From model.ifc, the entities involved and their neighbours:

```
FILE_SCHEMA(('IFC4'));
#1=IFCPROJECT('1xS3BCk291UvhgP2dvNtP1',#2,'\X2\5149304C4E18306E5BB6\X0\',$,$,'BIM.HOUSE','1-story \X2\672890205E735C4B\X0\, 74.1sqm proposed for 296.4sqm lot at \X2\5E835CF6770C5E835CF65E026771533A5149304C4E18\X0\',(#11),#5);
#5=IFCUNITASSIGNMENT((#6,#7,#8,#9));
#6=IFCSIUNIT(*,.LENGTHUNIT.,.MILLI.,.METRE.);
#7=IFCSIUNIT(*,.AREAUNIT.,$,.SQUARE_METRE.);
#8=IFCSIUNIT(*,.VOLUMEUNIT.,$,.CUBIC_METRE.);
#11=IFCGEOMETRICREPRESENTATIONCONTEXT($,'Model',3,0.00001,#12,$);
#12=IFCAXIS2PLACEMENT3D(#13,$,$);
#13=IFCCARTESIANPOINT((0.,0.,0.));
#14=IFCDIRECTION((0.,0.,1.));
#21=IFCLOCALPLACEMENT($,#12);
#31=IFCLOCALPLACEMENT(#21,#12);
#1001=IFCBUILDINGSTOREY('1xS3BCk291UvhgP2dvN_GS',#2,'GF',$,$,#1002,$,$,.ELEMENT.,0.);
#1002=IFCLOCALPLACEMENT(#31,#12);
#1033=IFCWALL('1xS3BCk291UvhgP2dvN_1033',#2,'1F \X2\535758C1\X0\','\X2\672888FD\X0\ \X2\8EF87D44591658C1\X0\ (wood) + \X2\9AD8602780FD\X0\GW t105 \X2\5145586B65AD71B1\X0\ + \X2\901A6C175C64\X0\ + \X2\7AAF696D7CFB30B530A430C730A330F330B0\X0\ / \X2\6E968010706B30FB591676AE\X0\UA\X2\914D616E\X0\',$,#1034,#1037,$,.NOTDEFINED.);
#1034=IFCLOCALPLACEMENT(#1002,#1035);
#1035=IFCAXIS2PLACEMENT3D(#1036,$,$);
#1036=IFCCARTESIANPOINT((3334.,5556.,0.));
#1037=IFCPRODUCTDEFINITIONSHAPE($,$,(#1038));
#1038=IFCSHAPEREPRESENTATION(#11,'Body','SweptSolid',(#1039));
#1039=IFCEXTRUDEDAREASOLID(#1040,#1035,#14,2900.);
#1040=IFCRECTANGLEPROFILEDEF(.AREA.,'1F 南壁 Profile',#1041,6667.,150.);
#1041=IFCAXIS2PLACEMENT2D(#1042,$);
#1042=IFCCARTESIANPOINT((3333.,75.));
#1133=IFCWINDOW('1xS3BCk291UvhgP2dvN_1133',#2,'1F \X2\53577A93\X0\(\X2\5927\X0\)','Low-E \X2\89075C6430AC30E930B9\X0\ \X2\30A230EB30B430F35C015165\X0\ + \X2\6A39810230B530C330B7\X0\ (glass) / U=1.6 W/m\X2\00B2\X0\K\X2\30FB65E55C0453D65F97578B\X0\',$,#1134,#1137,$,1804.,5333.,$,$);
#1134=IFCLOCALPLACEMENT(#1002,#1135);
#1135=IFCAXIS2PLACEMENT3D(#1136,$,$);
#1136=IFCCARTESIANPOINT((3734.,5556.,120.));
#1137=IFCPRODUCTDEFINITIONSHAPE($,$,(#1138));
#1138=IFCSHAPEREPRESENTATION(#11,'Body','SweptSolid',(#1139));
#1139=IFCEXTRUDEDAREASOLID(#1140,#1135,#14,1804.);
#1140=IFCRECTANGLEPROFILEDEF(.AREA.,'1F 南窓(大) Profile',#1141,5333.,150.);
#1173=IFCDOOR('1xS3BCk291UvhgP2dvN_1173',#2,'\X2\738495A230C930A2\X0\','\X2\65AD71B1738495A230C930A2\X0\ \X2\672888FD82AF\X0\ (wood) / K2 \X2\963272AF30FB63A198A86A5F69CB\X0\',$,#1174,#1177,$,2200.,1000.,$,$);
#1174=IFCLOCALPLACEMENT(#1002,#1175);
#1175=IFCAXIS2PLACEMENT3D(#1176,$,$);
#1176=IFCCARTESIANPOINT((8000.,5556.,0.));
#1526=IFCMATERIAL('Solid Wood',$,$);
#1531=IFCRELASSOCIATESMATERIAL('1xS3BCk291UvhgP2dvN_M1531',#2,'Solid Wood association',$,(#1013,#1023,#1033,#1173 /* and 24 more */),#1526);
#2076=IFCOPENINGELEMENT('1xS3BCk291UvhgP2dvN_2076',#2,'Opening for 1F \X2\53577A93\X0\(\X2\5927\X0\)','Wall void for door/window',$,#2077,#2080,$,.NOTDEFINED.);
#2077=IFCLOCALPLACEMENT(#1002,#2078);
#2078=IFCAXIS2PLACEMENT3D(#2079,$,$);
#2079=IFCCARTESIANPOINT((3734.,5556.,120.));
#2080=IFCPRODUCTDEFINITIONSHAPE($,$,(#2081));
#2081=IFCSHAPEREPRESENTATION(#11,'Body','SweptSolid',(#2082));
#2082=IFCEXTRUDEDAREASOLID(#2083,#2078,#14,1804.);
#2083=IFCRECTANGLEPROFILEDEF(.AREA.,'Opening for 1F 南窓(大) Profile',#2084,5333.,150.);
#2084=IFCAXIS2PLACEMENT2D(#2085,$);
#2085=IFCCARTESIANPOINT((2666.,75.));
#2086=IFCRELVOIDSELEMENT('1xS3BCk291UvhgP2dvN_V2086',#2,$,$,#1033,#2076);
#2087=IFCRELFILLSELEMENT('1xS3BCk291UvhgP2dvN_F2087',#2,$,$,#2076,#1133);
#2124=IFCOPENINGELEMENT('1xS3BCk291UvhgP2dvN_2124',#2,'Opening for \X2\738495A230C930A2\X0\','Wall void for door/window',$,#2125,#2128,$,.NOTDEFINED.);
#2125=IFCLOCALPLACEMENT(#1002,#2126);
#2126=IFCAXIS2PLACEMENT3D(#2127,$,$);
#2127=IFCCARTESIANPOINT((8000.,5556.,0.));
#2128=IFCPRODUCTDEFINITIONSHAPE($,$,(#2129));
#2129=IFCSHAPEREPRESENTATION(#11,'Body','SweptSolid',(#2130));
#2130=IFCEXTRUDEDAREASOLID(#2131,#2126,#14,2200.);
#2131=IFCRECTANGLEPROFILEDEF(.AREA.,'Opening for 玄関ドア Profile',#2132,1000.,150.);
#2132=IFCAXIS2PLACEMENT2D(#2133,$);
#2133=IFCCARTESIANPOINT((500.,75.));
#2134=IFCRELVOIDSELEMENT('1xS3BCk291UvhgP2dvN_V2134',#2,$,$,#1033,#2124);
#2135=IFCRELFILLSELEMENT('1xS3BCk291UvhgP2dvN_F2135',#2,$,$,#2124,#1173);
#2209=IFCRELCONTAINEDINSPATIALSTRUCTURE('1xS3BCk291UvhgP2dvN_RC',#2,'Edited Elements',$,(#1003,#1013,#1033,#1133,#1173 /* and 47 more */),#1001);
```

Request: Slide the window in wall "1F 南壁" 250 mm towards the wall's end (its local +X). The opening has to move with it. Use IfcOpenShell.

```python
import ifcopenshell
import ifcopenshell.api.geometry
import ifcopenshell.util.placement
import ifcopenshell.util.unit

model = ifcopenshell.open("model.ifc")
unit_scale = ifcopenshell.util.unit.calculate_unit_scale(model)

window = model.by_guid("1xS3BCk291UvhgP2dvN_1133")
opening = window.FillsVoids[0].RelatingOpeningElement
wall = opening.VoidsElements[0].RelatingBuildingElement

wall_matrix = ifcopenshell.util.placement.get_local_placement(wall.ObjectPlacement)
shift = wall_matrix[:3, 0] * 0.25 / unit_scale
before = ifcopenshell.util.placement.get_local_placement(window.ObjectPlacement)[:3, 3].copy()

# The window is not placed relative to its opening, so move both.
for product in (opening, window):
    matrix = ifcopenshell.util.placement.get_local_placement(product.ObjectPlacement)
    matrix[:3, 3] += shift
    ifcopenshell.api.geometry.edit_object_placement(model, product=product, matrix=matrix, is_si=False)

after = ifcopenshell.util.placement.get_local_placement(window.ObjectPlacement)[:3, 3]
print("window moved by", (after - before).round(3) + 0.0)

model.write("model_rev.ifc")
```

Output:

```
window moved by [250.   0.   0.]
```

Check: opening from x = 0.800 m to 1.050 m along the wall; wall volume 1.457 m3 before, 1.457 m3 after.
